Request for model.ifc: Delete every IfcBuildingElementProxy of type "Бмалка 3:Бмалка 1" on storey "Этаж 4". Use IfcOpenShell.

First a look at what the model holds.

```python
import ifcopenshell
import ifcopenshell.util.element

model = ifcopenshell.open("model.ifc")
print(model.schema)
storey = next(s for s in model.by_type("IfcBuildingStorey") if s.Name == "Этаж 4")
proxies = [e for e in ifcopenshell.util.element.get_decomposition(storey) if e.is_a("IfcBuildingElementProxy")]
seen = {}
for e in proxies:
    element_type = ifcopenshell.util.element.get_type(e)
    name = element_type.Name if element_type not in (None, e) else None
    seen[name] = seen.get(name, 0) + 1
for name, count in sorted(seen.items(), key=str):
    print(count, "x", name)
```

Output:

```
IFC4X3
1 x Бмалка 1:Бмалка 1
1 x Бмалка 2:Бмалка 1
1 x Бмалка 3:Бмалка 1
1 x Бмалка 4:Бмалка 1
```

```python
import ifcopenshell
import ifcopenshell.api.root
import ifcopenshell.util.element

model = ifcopenshell.open("model.ifc")

storey = next(s for s in model.by_type("IfcBuildingStorey") if s.Name == "Этаж 4")
proxies = [e for e in ifcopenshell.util.element.get_decomposition(storey) if e.is_a("IfcBuildingElementProxy")]
targets = [e for e in proxies if (t := ifcopenshell.util.element.get_type(e)) not in (None, e) and t.Name == "Бмалка 3:Бмалка 1"]

for e in targets:
    ifcopenshell.api.root.remove_product(model, product=e)
print(len(targets), "removed")

model.write("model_updated.ifc")
```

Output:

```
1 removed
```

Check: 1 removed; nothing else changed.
